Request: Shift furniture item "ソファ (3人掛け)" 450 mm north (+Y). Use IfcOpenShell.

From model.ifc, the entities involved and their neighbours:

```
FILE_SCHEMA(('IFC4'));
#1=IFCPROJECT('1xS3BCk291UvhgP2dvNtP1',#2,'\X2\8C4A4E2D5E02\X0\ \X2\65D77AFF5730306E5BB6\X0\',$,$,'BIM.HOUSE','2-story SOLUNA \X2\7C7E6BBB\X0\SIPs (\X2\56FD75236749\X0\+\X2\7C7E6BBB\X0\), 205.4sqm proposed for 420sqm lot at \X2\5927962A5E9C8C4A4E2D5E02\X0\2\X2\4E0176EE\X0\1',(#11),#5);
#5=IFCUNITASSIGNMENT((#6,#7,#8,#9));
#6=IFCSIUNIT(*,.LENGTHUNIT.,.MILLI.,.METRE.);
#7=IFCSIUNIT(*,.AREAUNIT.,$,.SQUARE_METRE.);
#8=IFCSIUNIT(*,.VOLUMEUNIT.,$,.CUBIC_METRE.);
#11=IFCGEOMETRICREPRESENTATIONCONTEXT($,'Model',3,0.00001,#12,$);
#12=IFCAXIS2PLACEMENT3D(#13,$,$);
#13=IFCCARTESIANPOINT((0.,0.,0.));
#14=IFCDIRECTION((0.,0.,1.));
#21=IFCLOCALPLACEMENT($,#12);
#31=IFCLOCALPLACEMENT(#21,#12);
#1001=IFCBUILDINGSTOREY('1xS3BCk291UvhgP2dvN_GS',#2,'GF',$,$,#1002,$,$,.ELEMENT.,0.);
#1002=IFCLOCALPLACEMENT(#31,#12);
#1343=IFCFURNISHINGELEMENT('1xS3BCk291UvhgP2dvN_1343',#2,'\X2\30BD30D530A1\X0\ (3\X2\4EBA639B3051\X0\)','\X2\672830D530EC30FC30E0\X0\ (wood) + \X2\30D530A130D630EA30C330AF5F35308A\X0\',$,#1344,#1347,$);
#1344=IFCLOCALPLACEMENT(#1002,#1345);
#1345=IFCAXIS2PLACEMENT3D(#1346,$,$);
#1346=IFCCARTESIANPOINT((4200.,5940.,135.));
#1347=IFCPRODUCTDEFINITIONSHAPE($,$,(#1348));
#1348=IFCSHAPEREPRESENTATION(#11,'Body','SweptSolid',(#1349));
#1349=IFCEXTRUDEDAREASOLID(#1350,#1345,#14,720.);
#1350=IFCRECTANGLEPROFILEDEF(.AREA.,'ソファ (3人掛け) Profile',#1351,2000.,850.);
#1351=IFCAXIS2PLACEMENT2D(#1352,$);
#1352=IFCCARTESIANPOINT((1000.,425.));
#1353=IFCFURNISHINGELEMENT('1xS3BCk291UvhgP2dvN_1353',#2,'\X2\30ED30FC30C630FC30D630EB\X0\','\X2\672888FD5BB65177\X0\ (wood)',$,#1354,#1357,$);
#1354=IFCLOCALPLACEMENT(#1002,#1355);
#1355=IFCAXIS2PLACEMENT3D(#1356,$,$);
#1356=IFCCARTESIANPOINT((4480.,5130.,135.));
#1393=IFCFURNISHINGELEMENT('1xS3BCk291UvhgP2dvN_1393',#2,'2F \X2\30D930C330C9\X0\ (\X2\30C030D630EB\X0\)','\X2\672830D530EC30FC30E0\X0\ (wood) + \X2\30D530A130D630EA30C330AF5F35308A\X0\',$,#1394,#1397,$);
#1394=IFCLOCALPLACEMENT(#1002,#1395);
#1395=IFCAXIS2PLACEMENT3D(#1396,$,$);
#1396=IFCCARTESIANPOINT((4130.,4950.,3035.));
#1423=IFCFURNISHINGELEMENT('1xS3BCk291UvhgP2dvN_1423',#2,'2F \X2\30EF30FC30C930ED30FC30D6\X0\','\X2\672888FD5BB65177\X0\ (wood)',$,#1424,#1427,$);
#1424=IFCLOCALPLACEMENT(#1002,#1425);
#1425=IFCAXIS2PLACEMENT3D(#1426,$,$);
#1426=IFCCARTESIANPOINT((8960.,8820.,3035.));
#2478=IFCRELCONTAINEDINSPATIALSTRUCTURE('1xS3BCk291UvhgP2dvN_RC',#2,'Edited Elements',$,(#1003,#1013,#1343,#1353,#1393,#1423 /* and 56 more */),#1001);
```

```python
import ifcopenshell
import ifcopenshell.api.geometry
import ifcopenshell.util.placement

model = ifcopenshell.open("model.ifc")

item = model.by_guid("1xS3BCk291UvhgP2dvN_1343")
matrix = ifcopenshell.util.placement.get_local_placement(item.ObjectPlacement)
matrix[1, 3] += 450.0
ifcopenshell.api.geometry.edit_object_placement(model, product=item, matrix=matrix, is_si=False)

print(ifcopenshell.util.placement.get_local_placement(item.ObjectPlacement).round(3) + 0.0)

model.write("model-out.ifc")
```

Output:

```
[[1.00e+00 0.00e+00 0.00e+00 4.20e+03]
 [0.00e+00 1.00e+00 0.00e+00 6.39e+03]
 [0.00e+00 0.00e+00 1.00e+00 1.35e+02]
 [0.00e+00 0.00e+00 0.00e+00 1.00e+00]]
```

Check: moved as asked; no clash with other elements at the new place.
